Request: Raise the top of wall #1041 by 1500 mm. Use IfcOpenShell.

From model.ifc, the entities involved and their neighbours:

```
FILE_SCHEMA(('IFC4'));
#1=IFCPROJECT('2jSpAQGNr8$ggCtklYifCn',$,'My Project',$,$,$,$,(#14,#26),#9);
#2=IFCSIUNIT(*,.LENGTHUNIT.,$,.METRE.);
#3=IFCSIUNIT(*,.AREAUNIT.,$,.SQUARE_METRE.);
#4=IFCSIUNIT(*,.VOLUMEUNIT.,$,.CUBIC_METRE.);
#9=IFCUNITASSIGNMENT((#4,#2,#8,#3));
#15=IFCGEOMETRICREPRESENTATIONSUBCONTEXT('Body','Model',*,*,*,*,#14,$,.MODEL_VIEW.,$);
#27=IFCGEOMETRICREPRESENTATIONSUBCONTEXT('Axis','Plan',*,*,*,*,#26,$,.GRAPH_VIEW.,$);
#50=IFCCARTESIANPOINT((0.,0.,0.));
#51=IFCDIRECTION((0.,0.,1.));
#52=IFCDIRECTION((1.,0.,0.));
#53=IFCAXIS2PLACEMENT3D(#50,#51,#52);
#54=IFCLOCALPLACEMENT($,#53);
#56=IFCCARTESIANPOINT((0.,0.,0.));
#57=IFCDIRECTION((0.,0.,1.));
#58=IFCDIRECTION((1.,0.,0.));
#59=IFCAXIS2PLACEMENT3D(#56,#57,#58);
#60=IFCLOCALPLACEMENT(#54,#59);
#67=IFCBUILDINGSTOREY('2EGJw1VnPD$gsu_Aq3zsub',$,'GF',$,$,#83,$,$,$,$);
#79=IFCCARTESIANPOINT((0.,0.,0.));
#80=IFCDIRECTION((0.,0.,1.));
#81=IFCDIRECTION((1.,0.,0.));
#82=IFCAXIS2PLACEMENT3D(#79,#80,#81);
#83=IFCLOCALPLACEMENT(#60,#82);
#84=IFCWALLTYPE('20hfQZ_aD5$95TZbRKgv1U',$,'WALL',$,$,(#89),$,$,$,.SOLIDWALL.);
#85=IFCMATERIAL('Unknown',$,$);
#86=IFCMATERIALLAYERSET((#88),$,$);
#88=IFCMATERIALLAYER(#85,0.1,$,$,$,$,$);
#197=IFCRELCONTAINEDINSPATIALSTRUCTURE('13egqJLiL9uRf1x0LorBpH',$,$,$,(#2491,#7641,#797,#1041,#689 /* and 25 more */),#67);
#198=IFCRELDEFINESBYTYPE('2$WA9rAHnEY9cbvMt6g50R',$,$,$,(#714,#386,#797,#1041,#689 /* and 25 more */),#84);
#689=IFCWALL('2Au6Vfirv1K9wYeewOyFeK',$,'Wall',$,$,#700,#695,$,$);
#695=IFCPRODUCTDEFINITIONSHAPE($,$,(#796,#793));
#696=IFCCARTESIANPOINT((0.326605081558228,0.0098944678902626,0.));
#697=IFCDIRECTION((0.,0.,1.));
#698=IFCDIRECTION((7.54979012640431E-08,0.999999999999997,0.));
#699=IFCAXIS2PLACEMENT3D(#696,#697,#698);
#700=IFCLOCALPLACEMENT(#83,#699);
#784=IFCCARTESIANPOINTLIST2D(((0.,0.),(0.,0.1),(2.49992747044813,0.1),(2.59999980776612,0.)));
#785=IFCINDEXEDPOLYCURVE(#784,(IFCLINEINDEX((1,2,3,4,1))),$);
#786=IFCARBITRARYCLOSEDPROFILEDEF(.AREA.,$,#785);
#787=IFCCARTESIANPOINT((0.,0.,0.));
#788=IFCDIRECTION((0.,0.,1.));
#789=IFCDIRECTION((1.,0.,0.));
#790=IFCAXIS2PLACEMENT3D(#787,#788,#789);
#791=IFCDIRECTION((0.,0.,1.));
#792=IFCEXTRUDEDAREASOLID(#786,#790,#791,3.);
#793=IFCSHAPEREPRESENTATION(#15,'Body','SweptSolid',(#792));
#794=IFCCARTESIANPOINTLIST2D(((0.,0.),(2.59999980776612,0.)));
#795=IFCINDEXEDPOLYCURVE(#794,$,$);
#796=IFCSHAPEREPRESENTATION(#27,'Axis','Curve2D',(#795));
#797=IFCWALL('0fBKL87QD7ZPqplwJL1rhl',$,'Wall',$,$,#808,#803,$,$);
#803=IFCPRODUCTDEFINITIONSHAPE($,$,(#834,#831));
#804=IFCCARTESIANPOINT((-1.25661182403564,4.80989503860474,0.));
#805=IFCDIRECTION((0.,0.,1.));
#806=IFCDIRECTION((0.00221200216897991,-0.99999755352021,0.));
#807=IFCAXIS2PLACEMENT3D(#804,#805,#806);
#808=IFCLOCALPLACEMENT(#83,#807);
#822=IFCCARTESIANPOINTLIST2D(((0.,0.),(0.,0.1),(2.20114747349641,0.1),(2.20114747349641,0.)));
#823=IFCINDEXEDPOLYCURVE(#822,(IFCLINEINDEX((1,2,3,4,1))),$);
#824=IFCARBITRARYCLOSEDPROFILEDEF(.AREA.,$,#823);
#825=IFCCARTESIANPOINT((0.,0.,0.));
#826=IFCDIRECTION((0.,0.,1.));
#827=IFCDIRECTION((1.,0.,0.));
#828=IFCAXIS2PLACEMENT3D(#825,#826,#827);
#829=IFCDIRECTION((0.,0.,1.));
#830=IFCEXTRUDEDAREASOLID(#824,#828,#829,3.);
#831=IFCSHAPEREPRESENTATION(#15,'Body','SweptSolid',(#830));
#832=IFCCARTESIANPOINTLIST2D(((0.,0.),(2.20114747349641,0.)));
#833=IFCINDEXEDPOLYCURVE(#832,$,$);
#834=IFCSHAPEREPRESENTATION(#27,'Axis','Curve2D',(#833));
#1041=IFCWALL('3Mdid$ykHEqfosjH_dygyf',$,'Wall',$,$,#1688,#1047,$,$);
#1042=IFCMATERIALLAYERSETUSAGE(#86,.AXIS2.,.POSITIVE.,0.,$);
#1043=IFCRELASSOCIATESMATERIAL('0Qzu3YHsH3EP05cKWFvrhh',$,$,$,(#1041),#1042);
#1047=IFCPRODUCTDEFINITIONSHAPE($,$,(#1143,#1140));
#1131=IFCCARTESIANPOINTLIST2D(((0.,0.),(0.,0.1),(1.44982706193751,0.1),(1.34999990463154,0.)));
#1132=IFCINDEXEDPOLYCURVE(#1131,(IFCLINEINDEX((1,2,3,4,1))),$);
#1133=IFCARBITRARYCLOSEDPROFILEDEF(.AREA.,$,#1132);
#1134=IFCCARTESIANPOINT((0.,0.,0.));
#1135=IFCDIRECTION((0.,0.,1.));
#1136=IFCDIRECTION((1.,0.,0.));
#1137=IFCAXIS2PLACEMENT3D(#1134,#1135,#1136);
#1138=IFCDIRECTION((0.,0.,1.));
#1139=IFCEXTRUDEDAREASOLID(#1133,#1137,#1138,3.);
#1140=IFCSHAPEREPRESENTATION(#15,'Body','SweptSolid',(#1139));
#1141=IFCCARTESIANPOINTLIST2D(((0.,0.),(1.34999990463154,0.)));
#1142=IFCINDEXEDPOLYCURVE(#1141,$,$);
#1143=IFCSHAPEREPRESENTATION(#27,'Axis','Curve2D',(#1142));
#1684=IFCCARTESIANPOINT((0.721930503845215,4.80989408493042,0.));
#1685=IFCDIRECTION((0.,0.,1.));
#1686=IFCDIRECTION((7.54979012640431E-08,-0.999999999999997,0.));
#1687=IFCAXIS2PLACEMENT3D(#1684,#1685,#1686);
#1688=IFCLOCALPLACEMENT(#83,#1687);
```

```python
import ifcopenshell
import ifcopenshell.geom
import ifcopenshell.util.representation
import ifcopenshell.util.shape

model = ifcopenshell.open("model.ifc")
settings = ifcopenshell.geom.settings()


def volume(element):
    """Net volume in cubic metres, openings subtracted."""
    shape = ifcopenshell.geom.create_shape(settings, element)
    return ifcopenshell.util.shape.get_volume(shape.geometry)


wall = model.by_guid("3Mdid$ykHEqfosjH_dygyf")
before = volume(wall)

body = ifcopenshell.util.representation.get_representation(wall, "Model", "Body")
solid = body.Items[0]
old_height = solid.Depth
solid.Depth += 1.5
after = volume(wall)

print(f"height {old_height:g} -> {solid.Depth:g}, volume {before:.3f} -> {after:.3f} m3")

model.write("model_edited.ifc")
```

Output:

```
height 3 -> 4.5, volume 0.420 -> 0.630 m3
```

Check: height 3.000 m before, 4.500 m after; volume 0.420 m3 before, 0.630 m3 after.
